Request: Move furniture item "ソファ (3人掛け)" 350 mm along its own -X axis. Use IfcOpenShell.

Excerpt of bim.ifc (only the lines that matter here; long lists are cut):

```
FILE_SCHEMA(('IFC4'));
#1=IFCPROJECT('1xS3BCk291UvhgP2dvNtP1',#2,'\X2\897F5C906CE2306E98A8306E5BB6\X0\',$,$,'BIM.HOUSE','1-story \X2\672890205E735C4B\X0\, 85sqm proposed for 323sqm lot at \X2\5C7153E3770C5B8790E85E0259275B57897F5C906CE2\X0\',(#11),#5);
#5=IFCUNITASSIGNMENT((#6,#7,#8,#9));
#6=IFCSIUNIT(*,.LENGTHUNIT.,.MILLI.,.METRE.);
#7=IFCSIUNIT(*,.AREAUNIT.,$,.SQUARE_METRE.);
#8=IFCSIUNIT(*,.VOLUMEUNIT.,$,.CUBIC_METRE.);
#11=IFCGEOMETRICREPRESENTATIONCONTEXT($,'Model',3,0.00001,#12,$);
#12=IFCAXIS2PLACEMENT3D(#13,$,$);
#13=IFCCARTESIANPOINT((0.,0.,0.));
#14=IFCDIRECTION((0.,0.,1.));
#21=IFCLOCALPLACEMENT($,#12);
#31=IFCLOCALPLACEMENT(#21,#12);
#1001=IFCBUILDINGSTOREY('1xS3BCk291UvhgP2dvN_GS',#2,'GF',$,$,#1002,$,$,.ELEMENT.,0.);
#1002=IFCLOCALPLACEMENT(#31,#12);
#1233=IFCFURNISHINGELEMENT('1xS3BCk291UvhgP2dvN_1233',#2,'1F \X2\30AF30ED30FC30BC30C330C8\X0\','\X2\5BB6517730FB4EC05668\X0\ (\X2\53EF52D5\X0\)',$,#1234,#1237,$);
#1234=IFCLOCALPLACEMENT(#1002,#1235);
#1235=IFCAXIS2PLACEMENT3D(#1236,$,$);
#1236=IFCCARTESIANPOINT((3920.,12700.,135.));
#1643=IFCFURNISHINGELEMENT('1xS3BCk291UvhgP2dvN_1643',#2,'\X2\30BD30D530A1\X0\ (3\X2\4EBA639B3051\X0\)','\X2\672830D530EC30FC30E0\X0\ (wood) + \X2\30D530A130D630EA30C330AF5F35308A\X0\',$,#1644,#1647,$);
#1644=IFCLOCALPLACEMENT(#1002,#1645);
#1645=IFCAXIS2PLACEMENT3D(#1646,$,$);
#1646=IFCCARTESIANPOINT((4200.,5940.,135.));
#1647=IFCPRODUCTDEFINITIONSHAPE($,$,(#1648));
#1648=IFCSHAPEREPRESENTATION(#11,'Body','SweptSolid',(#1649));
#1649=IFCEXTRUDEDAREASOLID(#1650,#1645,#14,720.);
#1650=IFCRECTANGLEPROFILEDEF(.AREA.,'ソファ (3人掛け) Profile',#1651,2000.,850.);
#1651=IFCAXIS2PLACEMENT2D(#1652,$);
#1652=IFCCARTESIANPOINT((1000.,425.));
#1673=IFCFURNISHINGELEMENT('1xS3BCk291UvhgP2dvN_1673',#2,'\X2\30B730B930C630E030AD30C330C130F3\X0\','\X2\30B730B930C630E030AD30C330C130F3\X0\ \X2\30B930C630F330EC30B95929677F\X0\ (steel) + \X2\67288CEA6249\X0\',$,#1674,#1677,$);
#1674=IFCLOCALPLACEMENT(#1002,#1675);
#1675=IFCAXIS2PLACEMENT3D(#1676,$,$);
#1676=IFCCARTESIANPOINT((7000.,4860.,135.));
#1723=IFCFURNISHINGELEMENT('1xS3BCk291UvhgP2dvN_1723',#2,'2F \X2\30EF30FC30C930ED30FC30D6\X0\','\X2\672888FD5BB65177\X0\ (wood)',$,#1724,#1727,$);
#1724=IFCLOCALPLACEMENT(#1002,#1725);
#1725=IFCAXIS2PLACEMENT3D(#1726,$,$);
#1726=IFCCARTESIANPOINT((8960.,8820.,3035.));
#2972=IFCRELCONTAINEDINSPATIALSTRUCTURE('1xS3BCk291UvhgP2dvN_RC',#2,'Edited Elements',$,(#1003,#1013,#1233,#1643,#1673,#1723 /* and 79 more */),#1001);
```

```python
import ifcopenshell
import ifcopenshell.api.geometry
import ifcopenshell.util.placement

model = ifcopenshell.open("bim.ifc")

item = model.by_id(1643)
matrix = ifcopenshell.util.placement.get_local_placement(item.ObjectPlacement)
matrix[:3, 3] -= matrix[:3, 0] * 350.0
ifcopenshell.api.geometry.edit_object_placement(model, product=item, matrix=matrix, is_si=False)

print(ifcopenshell.util.placement.get_local_placement(item.ObjectPlacement).round(3) + 0.0)

model.write("bim_rev.ifc")
```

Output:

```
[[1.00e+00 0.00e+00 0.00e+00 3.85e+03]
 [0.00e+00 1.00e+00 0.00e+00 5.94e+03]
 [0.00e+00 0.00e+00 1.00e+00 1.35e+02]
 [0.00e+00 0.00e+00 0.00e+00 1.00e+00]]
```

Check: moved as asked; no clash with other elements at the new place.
